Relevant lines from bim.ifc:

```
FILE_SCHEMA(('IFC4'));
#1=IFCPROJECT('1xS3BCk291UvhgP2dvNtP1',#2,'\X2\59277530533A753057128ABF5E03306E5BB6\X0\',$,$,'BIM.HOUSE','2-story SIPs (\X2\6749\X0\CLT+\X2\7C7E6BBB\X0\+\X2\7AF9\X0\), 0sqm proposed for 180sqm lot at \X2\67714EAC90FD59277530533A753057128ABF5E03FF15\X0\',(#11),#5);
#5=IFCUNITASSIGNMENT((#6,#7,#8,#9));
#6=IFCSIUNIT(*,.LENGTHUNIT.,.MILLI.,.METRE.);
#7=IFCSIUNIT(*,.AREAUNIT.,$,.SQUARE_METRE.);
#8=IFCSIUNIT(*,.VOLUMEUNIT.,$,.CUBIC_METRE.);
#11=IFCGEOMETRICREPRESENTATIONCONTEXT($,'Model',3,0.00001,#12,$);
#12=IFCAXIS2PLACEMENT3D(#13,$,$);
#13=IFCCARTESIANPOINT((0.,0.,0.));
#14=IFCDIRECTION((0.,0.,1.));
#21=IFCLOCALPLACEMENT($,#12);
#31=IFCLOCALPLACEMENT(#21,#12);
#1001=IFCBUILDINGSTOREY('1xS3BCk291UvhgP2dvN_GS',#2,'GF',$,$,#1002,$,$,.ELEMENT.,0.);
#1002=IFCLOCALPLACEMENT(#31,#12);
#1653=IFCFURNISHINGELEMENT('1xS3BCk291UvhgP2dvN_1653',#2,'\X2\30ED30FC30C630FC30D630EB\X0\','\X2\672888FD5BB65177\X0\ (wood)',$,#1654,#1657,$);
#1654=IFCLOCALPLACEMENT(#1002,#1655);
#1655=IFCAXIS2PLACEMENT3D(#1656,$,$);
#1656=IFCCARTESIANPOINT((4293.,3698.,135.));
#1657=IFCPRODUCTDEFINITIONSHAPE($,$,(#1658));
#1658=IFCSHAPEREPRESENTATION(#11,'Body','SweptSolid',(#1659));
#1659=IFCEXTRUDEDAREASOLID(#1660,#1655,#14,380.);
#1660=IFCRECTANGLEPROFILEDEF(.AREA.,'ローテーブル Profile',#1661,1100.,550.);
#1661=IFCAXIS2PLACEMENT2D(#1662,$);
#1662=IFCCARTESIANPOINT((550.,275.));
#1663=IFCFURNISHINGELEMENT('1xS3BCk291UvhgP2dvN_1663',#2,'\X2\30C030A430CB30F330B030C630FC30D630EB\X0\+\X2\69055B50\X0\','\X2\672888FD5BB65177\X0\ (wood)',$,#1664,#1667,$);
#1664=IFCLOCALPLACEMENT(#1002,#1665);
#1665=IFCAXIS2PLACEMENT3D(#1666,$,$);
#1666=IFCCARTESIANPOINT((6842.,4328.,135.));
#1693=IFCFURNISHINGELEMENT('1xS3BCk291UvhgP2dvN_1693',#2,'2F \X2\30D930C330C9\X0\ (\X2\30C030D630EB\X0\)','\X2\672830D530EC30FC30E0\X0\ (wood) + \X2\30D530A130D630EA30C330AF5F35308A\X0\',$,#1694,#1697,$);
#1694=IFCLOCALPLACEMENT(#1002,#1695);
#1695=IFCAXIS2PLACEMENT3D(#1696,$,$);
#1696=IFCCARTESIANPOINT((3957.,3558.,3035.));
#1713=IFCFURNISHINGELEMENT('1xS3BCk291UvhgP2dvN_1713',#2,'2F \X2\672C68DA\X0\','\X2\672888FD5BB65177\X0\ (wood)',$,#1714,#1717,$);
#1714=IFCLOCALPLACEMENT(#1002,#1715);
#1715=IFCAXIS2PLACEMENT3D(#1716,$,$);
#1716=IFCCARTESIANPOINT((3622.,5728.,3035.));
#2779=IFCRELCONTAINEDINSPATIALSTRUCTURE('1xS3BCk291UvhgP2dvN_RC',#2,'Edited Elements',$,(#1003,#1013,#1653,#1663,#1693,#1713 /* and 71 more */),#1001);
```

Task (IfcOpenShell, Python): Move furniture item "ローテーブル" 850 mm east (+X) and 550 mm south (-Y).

```python
import ifcopenshell
import ifcopenshell.api.geometry
import ifcopenshell.util.placement

model = ifcopenshell.open("bim.ifc")

item = model.by_guid("1xS3BCk291UvhgP2dvN_1653")
matrix = ifcopenshell.util.placement.get_local_placement(item.ObjectPlacement)
matrix[0, 3] += 850.0
matrix[1, 3] -= 550.0
ifcopenshell.api.geometry.edit_object_placement(model, product=item, matrix=matrix, is_si=False)

print(ifcopenshell.util.placement.get_local_placement(item.ObjectPlacement).round(3) + 0.0)

model.write("bim_rev.ifc")
```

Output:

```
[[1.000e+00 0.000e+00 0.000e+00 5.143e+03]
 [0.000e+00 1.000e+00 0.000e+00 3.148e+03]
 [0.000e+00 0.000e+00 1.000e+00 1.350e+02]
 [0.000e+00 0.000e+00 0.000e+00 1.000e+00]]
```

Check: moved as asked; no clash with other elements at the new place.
